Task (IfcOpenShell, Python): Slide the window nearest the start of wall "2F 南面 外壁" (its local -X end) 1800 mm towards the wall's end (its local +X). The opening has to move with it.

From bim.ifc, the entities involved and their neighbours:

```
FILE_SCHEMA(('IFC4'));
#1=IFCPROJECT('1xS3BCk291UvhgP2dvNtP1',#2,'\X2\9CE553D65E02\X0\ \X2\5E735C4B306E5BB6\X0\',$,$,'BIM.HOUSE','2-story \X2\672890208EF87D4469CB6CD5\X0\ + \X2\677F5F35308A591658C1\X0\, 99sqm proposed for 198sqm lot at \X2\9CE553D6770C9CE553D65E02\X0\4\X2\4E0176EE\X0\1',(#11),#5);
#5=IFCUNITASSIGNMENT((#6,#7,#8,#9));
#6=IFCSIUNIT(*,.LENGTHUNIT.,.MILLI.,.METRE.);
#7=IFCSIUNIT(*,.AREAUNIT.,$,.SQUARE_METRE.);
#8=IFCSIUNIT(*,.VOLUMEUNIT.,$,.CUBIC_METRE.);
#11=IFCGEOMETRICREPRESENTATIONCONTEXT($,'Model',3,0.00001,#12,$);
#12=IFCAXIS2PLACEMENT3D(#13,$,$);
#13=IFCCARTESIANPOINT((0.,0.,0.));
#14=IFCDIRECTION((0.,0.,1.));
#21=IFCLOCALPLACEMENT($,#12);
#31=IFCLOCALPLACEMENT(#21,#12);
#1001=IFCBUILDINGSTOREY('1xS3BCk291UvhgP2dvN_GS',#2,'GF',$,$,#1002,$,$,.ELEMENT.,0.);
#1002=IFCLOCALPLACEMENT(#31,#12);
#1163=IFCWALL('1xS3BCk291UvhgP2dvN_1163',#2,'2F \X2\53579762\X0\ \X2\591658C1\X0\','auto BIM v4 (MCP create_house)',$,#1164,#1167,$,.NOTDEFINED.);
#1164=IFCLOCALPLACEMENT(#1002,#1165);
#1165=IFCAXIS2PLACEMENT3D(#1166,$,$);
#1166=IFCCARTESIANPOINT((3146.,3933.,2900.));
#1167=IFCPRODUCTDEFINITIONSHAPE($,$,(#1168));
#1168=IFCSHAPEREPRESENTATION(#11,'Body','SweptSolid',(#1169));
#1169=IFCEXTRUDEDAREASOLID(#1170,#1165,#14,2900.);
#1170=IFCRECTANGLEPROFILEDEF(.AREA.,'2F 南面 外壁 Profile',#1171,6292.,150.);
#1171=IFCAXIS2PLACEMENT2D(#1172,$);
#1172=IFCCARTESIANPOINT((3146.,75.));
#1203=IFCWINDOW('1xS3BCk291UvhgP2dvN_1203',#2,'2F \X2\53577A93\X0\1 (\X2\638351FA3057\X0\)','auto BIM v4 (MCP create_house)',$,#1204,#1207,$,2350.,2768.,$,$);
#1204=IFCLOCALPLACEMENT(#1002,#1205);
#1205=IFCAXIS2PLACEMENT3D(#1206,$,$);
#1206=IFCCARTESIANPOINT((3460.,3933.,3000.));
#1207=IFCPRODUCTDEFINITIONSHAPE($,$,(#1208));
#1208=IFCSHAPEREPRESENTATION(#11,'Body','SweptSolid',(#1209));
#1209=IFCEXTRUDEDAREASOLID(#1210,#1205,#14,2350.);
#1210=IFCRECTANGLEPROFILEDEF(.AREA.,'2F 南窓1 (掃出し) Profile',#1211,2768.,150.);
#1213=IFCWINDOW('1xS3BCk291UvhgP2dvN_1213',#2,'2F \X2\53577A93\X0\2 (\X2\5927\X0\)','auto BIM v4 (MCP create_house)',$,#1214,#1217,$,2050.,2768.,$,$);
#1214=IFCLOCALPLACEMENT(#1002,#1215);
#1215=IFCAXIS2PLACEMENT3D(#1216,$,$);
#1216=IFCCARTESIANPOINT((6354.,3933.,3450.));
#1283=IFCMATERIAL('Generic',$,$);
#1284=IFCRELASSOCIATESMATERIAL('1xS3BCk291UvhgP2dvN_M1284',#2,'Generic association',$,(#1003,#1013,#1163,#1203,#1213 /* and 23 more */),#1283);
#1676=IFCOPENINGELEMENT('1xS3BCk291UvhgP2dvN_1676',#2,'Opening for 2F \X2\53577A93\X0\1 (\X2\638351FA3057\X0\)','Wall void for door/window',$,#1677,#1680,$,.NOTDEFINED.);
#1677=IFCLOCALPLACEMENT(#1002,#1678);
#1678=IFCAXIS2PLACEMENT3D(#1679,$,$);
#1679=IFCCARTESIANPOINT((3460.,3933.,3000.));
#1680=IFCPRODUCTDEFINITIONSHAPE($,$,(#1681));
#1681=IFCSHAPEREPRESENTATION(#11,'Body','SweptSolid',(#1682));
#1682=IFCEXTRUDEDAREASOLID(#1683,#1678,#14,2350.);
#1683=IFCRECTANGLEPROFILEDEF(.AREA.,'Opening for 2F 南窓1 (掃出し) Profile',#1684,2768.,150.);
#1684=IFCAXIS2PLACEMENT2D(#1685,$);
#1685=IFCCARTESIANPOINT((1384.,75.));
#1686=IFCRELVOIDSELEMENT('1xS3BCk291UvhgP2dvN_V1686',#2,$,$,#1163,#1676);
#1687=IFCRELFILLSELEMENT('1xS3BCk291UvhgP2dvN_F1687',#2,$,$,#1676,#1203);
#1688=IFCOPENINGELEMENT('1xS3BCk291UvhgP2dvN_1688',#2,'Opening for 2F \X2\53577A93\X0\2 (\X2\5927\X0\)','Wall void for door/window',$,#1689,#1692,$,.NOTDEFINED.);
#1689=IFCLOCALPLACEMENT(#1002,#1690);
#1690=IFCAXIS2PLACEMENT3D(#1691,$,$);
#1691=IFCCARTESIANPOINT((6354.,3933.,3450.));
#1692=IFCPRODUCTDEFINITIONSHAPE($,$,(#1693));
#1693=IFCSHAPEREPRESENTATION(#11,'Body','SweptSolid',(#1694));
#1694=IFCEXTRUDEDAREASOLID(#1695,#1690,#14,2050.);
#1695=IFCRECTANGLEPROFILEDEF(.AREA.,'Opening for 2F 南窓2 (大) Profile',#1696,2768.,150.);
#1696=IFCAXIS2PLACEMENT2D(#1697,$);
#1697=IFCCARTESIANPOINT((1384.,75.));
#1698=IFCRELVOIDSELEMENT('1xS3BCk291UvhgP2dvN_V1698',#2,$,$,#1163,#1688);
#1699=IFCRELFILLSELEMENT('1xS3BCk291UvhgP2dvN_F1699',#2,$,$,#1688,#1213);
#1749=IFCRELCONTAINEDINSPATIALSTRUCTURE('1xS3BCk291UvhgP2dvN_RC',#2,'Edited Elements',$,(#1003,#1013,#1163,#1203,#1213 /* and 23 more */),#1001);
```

```python
import ifcopenshell
import ifcopenshell.api.geometry
import ifcopenshell.util.placement

model = ifcopenshell.open("bim.ifc")

window = model.by_id(1203)
opening = window.FillsVoids[0].RelatingOpeningElement
wall = opening.VoidsElements[0].RelatingBuildingElement

wall_matrix = ifcopenshell.util.placement.get_local_placement(wall.ObjectPlacement)
shift = wall_matrix[:3, 0] * 1800.0
before = ifcopenshell.util.placement.get_local_placement(window.ObjectPlacement)[:3, 3].copy()

# The window is not placed relative to its opening, so move both.
for product in (opening, window):
    matrix = ifcopenshell.util.placement.get_local_placement(product.ObjectPlacement)
    matrix[:3, 3] += shift
    ifcopenshell.api.geometry.edit_object_placement(model, product=product, matrix=matrix, is_si=False)

after = ifcopenshell.util.placement.get_local_placement(window.ObjectPlacement)[:3, 3]
print("window moved by", (after - before).round(3) + 0.0)

model.write("bim_v2.ifc")
```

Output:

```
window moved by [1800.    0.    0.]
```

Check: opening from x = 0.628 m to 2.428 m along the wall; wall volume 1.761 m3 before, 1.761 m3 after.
